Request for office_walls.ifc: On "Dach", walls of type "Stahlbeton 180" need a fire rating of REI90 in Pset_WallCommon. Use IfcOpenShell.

First a look at what the model holds.

```python
import ifcopenshell
import ifcopenshell.util.element

model = ifcopenshell.open("office_walls.ifc")
print(model.schema)
storey = next(s for s in model.by_type("IfcBuildingStorey") if s.Name == "Dach")
walls = [e for e in ifcopenshell.util.element.get_decomposition(storey) if e.is_a("IfcWall")]
seen = {}
for e in walls:
    element_type = ifcopenshell.util.element.get_type(e)
    key = (element_type.Name if element_type != e and element_type else None, ifcopenshell.util.element.get_pset(e, "Pset_WallCommon", "FireRating"))
    seen[key] = seen.get(key, 0) + 1
for (name, value), count in sorted(seen.items(), key=str):
    print(count, "x", name, "|", value)
```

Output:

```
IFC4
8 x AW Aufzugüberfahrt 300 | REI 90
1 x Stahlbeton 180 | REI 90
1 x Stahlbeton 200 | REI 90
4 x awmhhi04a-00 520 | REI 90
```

```python
import ifcopenshell
import ifcopenshell.api.pset
import ifcopenshell.util.element

model = ifcopenshell.open("office_walls.ifc")

storey = next(s for s in model.by_type("IfcBuildingStorey") if s.Name == "Dach")
walls = [e for e in ifcopenshell.util.element.get_decomposition(storey) if e.is_a("IfcWall")]

count = 0
for e in walls:
    element_type = ifcopenshell.util.element.get_type(e)
    if element_type in (None, e) or element_type.Name != "Stahlbeton 180":
        continue
    # add_pset returns the element's existing set when there is one.
    pset = ifcopenshell.api.pset.add_pset(model, product=e, name="Pset_WallCommon")
    ifcopenshell.api.pset.edit_pset(model, pset=pset, properties={"FireRating": "REI90"})
    count += 1

print(count, "walls updated")

model.write("office_walls_edited.ifc")
```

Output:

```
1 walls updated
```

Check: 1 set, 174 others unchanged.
